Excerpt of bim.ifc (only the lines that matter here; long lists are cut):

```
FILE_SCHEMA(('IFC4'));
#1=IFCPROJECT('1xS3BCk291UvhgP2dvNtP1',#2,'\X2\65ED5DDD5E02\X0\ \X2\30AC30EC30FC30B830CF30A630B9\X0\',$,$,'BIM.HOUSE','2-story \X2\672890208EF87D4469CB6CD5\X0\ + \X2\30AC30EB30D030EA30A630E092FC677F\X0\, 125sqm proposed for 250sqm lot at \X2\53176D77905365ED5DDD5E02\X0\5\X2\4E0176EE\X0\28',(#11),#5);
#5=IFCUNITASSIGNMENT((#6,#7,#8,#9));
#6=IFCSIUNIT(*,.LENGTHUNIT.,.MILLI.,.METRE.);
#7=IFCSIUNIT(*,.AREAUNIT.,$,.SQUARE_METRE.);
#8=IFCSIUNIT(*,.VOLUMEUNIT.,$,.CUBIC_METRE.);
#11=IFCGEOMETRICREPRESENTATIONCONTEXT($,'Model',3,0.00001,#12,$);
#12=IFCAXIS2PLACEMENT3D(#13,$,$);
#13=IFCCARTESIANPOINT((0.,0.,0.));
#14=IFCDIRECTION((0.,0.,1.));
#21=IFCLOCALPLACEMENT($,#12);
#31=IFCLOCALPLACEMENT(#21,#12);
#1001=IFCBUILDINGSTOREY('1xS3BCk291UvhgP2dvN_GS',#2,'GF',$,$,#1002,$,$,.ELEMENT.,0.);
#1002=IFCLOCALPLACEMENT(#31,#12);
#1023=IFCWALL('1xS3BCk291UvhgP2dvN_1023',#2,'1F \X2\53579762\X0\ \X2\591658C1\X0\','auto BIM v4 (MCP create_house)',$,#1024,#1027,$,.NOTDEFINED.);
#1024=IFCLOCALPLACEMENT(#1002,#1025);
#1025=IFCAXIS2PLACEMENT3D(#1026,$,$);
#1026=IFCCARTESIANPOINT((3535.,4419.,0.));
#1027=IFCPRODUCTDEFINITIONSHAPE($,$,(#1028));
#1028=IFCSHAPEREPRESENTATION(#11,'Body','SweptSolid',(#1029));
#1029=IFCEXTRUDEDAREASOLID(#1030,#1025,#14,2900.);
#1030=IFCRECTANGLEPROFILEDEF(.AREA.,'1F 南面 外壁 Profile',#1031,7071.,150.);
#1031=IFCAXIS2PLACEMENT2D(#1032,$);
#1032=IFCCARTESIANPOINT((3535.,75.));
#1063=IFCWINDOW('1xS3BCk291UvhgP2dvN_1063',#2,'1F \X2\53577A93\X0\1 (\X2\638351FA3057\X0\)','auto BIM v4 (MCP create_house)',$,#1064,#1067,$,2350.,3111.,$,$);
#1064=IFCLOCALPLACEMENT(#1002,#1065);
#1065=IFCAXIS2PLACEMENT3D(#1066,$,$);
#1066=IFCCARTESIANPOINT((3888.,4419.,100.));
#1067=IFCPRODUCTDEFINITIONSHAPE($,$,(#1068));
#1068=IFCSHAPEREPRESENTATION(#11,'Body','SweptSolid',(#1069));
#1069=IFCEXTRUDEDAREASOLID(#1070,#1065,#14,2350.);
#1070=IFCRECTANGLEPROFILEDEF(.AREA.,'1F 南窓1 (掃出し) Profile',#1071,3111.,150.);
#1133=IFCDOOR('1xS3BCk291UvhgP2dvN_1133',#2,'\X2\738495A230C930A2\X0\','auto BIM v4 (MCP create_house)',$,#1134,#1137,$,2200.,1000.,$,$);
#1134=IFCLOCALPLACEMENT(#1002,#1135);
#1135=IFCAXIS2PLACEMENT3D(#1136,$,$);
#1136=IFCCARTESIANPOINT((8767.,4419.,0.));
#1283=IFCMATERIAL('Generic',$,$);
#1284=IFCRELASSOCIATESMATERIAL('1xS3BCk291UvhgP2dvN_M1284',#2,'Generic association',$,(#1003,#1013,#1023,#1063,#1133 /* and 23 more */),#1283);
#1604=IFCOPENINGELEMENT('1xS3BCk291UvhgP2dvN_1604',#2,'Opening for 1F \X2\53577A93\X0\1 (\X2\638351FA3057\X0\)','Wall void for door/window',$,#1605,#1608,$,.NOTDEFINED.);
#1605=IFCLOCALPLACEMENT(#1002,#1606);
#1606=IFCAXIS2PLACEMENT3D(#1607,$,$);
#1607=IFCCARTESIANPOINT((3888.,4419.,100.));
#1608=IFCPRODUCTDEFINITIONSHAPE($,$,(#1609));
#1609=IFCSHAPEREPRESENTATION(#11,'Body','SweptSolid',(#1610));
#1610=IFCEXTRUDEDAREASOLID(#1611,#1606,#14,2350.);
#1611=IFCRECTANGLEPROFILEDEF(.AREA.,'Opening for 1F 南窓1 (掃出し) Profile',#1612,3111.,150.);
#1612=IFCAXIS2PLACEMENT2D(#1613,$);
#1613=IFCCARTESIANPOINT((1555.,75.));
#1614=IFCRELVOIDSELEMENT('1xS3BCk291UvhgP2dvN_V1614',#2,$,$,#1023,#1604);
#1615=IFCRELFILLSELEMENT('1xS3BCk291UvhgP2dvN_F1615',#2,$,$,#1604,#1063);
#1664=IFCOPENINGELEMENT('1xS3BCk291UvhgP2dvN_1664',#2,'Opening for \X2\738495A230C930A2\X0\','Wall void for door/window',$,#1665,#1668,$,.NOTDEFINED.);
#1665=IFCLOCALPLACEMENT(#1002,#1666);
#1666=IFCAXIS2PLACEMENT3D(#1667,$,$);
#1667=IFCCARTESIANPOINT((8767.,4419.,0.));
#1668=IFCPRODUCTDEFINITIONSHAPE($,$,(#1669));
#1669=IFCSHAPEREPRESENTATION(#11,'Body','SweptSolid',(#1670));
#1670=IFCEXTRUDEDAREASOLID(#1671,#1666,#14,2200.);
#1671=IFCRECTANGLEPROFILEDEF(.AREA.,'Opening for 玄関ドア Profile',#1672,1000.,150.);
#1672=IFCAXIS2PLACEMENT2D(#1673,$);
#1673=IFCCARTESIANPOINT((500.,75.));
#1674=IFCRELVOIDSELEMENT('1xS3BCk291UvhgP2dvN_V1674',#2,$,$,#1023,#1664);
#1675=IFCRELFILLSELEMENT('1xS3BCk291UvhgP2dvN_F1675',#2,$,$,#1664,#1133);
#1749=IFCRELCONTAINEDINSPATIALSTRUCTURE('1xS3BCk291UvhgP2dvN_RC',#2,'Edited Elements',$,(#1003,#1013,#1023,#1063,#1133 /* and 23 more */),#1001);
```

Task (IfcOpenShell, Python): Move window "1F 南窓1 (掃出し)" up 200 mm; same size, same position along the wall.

```python
import numpy as np
import ifcopenshell
import ifcopenshell.api.geometry
import ifcopenshell.util.placement
import ifcopenshell.util.unit

model = ifcopenshell.open("bim.ifc")
unit_scale = ifcopenshell.util.unit.calculate_unit_scale(model)

window = model.by_guid("1xS3BCk291UvhgP2dvN_1063")
opening = window.FillsVoids[0].RelatingOpeningElement
dz = 200.0

shift = np.array([0.0, 0.0, dz])
# The window is not placed relative to its opening, so move both.
for product in (opening, window):
    matrix = ifcopenshell.util.placement.get_local_placement(product.ObjectPlacement)
    matrix[:3, 3] += shift
    ifcopenshell.api.geometry.edit_object_placement(model, product=product, matrix=matrix, is_si=False)

print(f"moved by {dz * unit_scale:+.3f} m")

model.write("bim-out.ifc")
```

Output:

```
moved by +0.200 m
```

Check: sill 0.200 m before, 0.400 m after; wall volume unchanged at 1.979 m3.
